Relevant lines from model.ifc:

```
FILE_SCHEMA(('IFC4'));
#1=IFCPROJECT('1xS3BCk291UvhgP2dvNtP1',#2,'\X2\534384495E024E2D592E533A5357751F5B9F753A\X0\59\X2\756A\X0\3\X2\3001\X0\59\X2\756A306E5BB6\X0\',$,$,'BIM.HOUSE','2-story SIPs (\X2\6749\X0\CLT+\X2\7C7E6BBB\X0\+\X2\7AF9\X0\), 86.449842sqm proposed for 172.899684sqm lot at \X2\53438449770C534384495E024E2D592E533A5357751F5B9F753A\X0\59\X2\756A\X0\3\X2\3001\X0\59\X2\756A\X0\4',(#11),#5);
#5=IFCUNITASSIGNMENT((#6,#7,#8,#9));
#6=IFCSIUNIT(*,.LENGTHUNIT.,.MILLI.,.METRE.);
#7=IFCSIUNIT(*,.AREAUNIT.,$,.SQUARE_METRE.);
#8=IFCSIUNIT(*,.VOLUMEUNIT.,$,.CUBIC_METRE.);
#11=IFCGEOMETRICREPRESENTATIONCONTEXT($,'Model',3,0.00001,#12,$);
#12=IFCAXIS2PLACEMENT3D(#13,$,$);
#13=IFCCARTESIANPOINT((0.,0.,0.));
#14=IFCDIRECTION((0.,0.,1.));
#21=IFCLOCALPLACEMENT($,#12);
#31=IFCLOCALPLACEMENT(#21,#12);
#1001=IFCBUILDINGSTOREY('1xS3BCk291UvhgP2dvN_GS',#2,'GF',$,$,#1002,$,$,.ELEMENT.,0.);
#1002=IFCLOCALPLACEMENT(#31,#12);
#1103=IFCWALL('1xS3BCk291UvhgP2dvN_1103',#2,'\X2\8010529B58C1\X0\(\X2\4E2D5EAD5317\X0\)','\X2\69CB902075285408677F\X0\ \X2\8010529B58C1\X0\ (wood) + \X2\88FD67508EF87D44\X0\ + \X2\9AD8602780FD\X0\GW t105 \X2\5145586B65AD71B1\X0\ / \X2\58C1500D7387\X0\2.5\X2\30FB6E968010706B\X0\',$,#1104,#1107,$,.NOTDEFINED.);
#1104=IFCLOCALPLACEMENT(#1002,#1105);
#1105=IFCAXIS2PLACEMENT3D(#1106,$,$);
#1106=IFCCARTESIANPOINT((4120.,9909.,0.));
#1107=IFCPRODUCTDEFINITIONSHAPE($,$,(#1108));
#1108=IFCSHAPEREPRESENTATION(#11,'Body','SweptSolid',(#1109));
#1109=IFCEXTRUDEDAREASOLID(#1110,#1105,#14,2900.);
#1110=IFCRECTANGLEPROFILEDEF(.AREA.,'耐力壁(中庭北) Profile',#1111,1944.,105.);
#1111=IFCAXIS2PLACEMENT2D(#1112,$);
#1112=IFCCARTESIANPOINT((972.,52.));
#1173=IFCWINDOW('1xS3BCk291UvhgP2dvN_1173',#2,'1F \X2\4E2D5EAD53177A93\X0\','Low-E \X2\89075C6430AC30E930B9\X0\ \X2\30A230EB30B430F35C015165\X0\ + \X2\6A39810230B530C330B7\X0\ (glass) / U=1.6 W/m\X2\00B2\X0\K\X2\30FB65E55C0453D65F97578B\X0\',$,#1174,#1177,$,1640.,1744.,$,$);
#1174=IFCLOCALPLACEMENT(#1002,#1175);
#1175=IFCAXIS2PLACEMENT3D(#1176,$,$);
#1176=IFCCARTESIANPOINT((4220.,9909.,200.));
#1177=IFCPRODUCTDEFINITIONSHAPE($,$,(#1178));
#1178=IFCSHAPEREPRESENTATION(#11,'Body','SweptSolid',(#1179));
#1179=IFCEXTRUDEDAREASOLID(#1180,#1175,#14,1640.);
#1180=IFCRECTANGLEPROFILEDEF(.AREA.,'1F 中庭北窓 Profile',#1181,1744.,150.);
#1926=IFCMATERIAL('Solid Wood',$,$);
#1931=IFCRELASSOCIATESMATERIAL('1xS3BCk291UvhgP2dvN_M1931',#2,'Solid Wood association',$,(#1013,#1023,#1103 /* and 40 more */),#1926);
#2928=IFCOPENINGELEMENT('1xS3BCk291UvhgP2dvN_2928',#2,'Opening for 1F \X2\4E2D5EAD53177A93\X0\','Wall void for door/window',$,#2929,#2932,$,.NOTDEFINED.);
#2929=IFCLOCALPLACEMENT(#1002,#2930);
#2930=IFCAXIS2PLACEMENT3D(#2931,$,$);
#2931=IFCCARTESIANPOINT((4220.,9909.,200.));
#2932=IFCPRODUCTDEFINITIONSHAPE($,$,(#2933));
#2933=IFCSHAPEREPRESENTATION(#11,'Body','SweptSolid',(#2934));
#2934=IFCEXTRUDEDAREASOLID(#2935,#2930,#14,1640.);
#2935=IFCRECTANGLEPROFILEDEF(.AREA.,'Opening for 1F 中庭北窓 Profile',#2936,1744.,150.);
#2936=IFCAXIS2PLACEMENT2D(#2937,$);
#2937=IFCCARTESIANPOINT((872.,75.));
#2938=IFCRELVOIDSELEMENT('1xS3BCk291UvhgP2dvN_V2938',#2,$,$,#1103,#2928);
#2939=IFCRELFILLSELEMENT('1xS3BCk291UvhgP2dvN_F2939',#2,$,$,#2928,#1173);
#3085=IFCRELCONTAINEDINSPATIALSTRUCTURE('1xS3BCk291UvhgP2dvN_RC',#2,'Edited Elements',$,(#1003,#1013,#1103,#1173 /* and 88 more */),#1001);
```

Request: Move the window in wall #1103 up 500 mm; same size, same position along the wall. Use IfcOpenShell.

```python
import numpy as np
import ifcopenshell
import ifcopenshell.api.geometry
import ifcopenshell.util.placement
import ifcopenshell.util.unit

model = ifcopenshell.open("model.ifc")
unit_scale = ifcopenshell.util.unit.calculate_unit_scale(model)

window = model.by_guid("1xS3BCk291UvhgP2dvN_1173")
opening = window.FillsVoids[0].RelatingOpeningElement
dz = 0.5 / unit_scale

shift = np.array([0.0, 0.0, dz])
# The window is not placed relative to its opening, so move both.
for product in (opening, window):
    matrix = ifcopenshell.util.placement.get_local_placement(product.ObjectPlacement)
    matrix[:3, 3] += shift
    ifcopenshell.api.geometry.edit_object_placement(model, product=product, matrix=matrix, is_si=False)

print(f"moved by {dz * unit_scale:+.3f} m")

model.write("model_rev.ifc")
```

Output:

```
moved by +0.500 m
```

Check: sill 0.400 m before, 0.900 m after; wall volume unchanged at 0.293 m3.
